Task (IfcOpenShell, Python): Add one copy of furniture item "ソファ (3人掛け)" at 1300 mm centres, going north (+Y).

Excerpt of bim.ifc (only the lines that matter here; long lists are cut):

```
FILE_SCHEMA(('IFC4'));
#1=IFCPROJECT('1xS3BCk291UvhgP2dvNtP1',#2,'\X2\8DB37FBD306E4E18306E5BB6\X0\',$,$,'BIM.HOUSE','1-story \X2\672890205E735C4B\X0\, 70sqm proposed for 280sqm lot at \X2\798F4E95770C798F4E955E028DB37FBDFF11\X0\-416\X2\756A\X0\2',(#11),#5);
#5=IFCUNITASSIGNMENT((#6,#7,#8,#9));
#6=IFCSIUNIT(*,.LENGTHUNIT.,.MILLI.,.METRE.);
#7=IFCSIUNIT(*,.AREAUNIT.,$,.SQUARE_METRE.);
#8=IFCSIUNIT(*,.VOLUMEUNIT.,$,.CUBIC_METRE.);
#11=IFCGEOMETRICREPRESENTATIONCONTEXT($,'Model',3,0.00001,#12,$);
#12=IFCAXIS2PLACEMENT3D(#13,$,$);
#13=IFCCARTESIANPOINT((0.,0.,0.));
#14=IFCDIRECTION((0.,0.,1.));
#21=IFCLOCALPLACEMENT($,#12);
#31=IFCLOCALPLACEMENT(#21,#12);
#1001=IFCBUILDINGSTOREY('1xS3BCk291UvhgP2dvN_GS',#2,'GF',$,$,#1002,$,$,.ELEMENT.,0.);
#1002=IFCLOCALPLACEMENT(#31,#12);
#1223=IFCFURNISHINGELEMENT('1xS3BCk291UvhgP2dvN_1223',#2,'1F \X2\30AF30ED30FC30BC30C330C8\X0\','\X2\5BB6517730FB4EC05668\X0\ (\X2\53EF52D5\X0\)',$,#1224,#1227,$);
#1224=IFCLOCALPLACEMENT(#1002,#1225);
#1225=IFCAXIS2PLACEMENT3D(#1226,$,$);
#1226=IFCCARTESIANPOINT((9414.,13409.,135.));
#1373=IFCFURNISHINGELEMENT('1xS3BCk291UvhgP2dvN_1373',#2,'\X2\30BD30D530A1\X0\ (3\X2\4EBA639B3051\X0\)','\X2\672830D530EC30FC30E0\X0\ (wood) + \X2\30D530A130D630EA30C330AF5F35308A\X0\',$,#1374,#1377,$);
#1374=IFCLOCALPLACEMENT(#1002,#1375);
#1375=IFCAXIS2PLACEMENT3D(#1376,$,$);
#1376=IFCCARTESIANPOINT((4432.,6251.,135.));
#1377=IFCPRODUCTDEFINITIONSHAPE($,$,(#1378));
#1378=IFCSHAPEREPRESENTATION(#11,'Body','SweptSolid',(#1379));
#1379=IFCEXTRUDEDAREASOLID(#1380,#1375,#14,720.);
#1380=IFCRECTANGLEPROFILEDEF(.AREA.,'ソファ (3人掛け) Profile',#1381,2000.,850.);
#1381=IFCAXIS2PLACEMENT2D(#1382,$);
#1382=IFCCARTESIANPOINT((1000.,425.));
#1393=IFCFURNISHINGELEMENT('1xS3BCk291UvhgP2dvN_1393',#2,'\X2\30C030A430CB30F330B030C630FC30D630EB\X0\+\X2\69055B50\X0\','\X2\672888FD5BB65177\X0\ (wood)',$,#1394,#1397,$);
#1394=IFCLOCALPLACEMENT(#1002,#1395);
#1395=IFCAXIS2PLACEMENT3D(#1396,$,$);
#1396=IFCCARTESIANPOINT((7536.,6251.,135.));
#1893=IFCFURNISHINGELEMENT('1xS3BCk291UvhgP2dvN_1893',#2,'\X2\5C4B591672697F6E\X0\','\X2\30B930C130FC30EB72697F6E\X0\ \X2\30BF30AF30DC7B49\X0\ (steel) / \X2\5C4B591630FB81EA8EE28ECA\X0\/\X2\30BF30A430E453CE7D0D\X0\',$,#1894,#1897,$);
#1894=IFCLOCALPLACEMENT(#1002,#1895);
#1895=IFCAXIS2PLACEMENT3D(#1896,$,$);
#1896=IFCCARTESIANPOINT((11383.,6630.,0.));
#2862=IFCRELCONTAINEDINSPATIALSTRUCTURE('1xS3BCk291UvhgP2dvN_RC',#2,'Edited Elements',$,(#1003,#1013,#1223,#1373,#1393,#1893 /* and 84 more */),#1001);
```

```python
import numpy as np
import ifcopenshell
import ifcopenshell.api.geometry
import ifcopenshell.api.root
import ifcopenshell.util.element
import ifcopenshell.util.placement

model = ifcopenshell.open("bim.ifc")


def reuse_history(source, copy):
    """copy_class also copies each property set's owner history, people and application; keep the originals."""
    for rel in copy.IsDefinedBy:
        if rel.is_a("IfcRelDefinesByProperties") and (history := rel.RelatingPropertyDefinition.OwnerHistory):
            rel.RelatingPropertyDefinition.OwnerHistory = source.OwnerHistory
            ifcopenshell.util.element.remove_deep2(model, history)


source = model.by_guid("1xS3BCk291UvhgP2dvN_1373")
base = ifcopenshell.util.placement.get_local_placement(source.ObjectPlacement)
step = np.array([0.0, 1.0, 0.0]) * 1300.0

for i in range(1, 2):
    copy = ifcopenshell.api.root.copy_class(model, product=source)
    copy.Representation = ifcopenshell.util.element.copy_deep(
        model, source.Representation, exclude=["IfcGeometricRepresentationContext", "IfcRepresentationMap"]
    )
    reuse_history(source, copy)
    matrix = base.copy()
    matrix[:3, 3] += i * step
    print("added at", matrix[:3, 3].round(3) + 0.0)
    ifcopenshell.api.geometry.edit_object_placement(model, product=copy, matrix=matrix, is_si=False)

model.write("bim_updated.ifc")
```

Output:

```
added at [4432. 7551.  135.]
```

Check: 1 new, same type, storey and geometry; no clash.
